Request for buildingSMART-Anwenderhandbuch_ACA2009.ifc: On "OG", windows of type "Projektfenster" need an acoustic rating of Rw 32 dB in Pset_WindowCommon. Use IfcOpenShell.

First a look at what the model holds.

```python
import ifcopenshell
import ifcopenshell.util.element

model = ifcopenshell.open("buildingSMART-Anwenderhandbuch_ACA2009.ifc")
print(model.schema)
storey = next(s for s in model.by_type("IfcBuildingStorey") if s.Name == "OG")
windows = [e for e in ifcopenshell.util.element.get_decomposition(storey) if e.is_a("IfcWindow")]
seen = {}
for e in windows:
    element_type = ifcopenshell.util.element.get_type(e)
    key = (element_type.Name if element_type != e and element_type else None, ifcopenshell.util.element.get_pset(e, "Pset_WindowCommon", "AcousticRating"))
    seen[key] = seen.get(key, 0) + 1
for (name, value), count in sorted(seen.items(), key=str):
    print(count, "x", name, "|", value)
```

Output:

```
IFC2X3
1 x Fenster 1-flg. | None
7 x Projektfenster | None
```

```python
import ifcopenshell
import ifcopenshell.api.pset
import ifcopenshell.util.element

model = ifcopenshell.open("buildingSMART-Anwenderhandbuch_ACA2009.ifc")

storey = next(s for s in model.by_type("IfcBuildingStorey") if s.Name == "OG")
windows = [e for e in ifcopenshell.util.element.get_decomposition(storey) if e.is_a("IfcWindow")]

count = 0
for e in windows:
    element_type = ifcopenshell.util.element.get_type(e)
    if element_type in (None, e) or element_type.Name != "Projektfenster":
        continue
    # add_pset returns the element's existing set when there is one.
    pset = ifcopenshell.api.pset.add_pset(model, product=e, name="Pset_WindowCommon")
    ifcopenshell.api.pset.edit_pset(model, pset=pset, properties={"AcousticRating": "Rw 32 dB"})
    count += 1

print(count, "windows updated")

model.write("buildingSMART-Anwenderhandbuch_ACA2009-out.ifc")
```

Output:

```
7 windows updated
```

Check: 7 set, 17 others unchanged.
